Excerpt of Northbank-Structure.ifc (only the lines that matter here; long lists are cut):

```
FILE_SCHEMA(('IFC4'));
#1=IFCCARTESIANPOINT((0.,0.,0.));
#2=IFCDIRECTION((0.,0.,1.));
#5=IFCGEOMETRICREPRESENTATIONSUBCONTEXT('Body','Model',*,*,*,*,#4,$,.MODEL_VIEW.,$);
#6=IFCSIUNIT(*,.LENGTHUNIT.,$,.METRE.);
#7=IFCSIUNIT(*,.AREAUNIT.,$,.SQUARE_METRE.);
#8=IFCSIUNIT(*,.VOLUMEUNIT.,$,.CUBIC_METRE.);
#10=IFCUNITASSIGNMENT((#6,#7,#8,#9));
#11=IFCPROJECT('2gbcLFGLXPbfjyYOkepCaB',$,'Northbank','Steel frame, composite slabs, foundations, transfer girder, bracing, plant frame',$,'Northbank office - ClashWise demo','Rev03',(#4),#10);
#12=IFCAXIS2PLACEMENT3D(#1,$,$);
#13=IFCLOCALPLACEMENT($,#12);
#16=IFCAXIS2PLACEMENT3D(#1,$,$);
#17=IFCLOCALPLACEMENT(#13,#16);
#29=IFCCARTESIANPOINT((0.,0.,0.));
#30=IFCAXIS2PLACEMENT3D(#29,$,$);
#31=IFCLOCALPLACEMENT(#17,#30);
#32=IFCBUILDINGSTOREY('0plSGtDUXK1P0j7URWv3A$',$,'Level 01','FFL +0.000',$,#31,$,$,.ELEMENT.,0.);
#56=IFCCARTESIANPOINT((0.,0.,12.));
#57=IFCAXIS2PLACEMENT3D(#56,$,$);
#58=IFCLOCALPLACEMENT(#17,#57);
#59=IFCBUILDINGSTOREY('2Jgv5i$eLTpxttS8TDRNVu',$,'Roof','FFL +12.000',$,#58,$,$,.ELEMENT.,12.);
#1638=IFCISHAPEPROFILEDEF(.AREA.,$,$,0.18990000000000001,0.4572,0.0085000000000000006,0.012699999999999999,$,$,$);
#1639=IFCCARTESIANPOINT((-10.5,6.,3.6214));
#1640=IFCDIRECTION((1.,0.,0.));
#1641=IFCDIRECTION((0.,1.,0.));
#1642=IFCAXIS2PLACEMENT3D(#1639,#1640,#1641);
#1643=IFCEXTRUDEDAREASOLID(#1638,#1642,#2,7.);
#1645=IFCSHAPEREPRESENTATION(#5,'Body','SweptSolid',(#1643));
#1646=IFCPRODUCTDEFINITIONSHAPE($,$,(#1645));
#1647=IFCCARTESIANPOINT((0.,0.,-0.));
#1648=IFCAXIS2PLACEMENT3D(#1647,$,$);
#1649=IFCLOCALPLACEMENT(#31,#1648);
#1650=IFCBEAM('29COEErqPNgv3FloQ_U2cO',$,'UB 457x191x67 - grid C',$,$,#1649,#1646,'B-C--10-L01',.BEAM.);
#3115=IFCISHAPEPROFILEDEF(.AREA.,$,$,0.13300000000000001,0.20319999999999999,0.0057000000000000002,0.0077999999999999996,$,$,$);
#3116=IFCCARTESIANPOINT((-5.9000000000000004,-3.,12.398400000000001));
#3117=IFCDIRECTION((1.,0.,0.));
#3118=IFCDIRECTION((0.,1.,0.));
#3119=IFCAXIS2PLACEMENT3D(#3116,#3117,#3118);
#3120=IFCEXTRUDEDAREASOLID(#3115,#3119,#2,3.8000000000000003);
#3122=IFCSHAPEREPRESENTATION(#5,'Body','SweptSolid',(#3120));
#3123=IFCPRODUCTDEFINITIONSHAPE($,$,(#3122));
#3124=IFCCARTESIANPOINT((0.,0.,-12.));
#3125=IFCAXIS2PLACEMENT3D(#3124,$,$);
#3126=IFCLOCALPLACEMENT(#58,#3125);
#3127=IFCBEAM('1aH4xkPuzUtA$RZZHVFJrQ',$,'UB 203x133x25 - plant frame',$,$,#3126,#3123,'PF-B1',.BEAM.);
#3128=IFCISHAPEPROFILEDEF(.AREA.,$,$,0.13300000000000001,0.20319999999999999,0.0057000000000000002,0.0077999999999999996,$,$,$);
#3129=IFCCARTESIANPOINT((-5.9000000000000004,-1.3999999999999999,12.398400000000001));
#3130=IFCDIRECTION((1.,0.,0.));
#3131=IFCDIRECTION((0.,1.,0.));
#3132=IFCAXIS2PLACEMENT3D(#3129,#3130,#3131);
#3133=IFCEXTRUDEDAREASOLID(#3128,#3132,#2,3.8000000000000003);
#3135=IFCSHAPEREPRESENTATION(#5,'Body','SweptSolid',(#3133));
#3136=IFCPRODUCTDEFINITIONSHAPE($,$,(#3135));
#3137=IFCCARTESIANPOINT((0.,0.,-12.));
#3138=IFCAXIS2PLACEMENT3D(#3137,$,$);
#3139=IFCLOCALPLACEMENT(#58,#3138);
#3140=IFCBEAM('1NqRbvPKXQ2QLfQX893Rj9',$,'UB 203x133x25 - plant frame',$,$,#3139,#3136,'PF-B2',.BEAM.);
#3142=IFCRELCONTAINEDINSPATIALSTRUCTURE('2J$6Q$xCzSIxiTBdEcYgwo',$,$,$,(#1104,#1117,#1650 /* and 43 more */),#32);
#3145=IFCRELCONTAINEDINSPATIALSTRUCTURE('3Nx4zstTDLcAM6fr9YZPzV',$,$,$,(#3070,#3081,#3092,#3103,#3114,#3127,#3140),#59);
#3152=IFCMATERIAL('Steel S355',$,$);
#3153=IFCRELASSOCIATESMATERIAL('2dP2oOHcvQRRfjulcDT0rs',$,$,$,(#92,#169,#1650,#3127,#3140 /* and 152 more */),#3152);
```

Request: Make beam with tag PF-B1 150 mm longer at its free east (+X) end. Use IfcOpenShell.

```python
import ifcopenshell
import ifcopenshell.util.representation
import ifcopenshell.util.unit

model = ifcopenshell.open("Northbank-Structure.ifc")
unit_scale = ifcopenshell.util.unit.calculate_unit_scale(model)

member = model.by_guid("1aH4xkPuzUtA$RZZHVFJrQ")
change = 0.15 / unit_scale

# The extrusion runs towards the end named, so only its depth changes.
body = ifcopenshell.util.representation.get_representation(member, "Model", "Body")
solid = body.Items[0]
old_length = solid.Depth
solid.Depth += change

print(f"length {old_length:g} -> {solid.Depth:g}")

model.write("Northbank-Structure_v2.ifc")
```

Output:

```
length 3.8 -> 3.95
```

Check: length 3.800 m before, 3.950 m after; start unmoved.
